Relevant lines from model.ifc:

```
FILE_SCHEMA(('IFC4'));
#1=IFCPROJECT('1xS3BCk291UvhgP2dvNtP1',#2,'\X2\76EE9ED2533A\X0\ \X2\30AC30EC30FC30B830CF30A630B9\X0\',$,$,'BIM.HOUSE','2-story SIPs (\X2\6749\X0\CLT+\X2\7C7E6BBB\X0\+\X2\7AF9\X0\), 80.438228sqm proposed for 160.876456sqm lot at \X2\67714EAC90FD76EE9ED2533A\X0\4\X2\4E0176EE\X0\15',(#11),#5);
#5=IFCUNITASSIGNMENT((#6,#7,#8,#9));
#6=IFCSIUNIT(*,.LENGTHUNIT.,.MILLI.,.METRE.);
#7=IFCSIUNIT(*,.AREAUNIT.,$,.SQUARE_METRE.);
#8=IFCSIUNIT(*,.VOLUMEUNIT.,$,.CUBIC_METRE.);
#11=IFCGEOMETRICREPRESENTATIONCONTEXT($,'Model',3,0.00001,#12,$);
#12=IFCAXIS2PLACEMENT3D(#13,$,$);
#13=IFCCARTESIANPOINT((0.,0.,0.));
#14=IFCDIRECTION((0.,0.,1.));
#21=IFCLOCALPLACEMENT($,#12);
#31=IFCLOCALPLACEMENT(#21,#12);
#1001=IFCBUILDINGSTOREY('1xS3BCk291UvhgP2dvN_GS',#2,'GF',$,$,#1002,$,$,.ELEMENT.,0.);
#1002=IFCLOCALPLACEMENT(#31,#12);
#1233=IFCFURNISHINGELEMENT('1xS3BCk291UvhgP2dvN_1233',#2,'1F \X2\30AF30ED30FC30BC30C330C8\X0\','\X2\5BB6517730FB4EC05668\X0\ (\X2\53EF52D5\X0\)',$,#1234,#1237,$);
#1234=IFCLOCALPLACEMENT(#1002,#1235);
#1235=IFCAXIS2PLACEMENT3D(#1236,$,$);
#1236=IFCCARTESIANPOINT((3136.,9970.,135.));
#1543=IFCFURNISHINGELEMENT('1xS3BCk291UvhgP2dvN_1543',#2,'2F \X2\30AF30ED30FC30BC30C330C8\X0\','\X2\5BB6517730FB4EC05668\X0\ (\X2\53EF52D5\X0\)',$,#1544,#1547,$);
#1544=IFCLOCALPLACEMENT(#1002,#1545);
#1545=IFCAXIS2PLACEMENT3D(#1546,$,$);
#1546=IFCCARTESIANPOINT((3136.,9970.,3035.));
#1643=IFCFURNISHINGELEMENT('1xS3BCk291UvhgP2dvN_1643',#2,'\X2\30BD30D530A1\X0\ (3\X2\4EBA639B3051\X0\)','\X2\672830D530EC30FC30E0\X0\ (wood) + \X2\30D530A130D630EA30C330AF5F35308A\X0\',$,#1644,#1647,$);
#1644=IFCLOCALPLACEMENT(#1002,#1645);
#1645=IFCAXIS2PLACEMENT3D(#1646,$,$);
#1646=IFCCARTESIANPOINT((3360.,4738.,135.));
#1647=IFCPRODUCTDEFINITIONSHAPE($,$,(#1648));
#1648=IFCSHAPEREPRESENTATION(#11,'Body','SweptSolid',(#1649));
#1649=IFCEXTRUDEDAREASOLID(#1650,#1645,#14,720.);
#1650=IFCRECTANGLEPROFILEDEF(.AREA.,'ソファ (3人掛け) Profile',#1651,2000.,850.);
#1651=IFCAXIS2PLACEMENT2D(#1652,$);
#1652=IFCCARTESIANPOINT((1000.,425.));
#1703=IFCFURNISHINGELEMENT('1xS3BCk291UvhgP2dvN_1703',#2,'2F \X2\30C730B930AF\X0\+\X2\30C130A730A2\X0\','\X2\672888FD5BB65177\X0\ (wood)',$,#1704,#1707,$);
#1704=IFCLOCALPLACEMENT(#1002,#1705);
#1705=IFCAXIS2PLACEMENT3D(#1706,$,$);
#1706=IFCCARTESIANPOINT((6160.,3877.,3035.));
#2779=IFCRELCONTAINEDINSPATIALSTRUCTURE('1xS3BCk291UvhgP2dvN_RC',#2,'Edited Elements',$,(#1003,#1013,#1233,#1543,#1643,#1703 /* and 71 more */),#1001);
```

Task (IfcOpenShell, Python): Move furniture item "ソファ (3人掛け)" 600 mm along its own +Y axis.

```python
import ifcopenshell
import ifcopenshell.api.geometry
import ifcopenshell.util.placement
import ifcopenshell.util.unit

model = ifcopenshell.open("model.ifc")
unit_scale = ifcopenshell.util.unit.calculate_unit_scale(model)

item = model.by_guid("1xS3BCk291UvhgP2dvN_1643")
matrix = ifcopenshell.util.placement.get_local_placement(item.ObjectPlacement)
matrix[:3, 3] += matrix[:3, 1] * 0.6 / unit_scale
ifcopenshell.api.geometry.edit_object_placement(model, product=item, matrix=matrix, is_si=False)

print(ifcopenshell.util.placement.get_local_placement(item.ObjectPlacement).round(3) + 0.0)

model.write("model_rev.ifc")
```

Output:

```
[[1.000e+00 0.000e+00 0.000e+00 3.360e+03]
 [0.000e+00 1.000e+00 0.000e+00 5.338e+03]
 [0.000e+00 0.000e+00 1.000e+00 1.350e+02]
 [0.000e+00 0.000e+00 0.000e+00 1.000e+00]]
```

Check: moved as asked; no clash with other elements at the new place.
